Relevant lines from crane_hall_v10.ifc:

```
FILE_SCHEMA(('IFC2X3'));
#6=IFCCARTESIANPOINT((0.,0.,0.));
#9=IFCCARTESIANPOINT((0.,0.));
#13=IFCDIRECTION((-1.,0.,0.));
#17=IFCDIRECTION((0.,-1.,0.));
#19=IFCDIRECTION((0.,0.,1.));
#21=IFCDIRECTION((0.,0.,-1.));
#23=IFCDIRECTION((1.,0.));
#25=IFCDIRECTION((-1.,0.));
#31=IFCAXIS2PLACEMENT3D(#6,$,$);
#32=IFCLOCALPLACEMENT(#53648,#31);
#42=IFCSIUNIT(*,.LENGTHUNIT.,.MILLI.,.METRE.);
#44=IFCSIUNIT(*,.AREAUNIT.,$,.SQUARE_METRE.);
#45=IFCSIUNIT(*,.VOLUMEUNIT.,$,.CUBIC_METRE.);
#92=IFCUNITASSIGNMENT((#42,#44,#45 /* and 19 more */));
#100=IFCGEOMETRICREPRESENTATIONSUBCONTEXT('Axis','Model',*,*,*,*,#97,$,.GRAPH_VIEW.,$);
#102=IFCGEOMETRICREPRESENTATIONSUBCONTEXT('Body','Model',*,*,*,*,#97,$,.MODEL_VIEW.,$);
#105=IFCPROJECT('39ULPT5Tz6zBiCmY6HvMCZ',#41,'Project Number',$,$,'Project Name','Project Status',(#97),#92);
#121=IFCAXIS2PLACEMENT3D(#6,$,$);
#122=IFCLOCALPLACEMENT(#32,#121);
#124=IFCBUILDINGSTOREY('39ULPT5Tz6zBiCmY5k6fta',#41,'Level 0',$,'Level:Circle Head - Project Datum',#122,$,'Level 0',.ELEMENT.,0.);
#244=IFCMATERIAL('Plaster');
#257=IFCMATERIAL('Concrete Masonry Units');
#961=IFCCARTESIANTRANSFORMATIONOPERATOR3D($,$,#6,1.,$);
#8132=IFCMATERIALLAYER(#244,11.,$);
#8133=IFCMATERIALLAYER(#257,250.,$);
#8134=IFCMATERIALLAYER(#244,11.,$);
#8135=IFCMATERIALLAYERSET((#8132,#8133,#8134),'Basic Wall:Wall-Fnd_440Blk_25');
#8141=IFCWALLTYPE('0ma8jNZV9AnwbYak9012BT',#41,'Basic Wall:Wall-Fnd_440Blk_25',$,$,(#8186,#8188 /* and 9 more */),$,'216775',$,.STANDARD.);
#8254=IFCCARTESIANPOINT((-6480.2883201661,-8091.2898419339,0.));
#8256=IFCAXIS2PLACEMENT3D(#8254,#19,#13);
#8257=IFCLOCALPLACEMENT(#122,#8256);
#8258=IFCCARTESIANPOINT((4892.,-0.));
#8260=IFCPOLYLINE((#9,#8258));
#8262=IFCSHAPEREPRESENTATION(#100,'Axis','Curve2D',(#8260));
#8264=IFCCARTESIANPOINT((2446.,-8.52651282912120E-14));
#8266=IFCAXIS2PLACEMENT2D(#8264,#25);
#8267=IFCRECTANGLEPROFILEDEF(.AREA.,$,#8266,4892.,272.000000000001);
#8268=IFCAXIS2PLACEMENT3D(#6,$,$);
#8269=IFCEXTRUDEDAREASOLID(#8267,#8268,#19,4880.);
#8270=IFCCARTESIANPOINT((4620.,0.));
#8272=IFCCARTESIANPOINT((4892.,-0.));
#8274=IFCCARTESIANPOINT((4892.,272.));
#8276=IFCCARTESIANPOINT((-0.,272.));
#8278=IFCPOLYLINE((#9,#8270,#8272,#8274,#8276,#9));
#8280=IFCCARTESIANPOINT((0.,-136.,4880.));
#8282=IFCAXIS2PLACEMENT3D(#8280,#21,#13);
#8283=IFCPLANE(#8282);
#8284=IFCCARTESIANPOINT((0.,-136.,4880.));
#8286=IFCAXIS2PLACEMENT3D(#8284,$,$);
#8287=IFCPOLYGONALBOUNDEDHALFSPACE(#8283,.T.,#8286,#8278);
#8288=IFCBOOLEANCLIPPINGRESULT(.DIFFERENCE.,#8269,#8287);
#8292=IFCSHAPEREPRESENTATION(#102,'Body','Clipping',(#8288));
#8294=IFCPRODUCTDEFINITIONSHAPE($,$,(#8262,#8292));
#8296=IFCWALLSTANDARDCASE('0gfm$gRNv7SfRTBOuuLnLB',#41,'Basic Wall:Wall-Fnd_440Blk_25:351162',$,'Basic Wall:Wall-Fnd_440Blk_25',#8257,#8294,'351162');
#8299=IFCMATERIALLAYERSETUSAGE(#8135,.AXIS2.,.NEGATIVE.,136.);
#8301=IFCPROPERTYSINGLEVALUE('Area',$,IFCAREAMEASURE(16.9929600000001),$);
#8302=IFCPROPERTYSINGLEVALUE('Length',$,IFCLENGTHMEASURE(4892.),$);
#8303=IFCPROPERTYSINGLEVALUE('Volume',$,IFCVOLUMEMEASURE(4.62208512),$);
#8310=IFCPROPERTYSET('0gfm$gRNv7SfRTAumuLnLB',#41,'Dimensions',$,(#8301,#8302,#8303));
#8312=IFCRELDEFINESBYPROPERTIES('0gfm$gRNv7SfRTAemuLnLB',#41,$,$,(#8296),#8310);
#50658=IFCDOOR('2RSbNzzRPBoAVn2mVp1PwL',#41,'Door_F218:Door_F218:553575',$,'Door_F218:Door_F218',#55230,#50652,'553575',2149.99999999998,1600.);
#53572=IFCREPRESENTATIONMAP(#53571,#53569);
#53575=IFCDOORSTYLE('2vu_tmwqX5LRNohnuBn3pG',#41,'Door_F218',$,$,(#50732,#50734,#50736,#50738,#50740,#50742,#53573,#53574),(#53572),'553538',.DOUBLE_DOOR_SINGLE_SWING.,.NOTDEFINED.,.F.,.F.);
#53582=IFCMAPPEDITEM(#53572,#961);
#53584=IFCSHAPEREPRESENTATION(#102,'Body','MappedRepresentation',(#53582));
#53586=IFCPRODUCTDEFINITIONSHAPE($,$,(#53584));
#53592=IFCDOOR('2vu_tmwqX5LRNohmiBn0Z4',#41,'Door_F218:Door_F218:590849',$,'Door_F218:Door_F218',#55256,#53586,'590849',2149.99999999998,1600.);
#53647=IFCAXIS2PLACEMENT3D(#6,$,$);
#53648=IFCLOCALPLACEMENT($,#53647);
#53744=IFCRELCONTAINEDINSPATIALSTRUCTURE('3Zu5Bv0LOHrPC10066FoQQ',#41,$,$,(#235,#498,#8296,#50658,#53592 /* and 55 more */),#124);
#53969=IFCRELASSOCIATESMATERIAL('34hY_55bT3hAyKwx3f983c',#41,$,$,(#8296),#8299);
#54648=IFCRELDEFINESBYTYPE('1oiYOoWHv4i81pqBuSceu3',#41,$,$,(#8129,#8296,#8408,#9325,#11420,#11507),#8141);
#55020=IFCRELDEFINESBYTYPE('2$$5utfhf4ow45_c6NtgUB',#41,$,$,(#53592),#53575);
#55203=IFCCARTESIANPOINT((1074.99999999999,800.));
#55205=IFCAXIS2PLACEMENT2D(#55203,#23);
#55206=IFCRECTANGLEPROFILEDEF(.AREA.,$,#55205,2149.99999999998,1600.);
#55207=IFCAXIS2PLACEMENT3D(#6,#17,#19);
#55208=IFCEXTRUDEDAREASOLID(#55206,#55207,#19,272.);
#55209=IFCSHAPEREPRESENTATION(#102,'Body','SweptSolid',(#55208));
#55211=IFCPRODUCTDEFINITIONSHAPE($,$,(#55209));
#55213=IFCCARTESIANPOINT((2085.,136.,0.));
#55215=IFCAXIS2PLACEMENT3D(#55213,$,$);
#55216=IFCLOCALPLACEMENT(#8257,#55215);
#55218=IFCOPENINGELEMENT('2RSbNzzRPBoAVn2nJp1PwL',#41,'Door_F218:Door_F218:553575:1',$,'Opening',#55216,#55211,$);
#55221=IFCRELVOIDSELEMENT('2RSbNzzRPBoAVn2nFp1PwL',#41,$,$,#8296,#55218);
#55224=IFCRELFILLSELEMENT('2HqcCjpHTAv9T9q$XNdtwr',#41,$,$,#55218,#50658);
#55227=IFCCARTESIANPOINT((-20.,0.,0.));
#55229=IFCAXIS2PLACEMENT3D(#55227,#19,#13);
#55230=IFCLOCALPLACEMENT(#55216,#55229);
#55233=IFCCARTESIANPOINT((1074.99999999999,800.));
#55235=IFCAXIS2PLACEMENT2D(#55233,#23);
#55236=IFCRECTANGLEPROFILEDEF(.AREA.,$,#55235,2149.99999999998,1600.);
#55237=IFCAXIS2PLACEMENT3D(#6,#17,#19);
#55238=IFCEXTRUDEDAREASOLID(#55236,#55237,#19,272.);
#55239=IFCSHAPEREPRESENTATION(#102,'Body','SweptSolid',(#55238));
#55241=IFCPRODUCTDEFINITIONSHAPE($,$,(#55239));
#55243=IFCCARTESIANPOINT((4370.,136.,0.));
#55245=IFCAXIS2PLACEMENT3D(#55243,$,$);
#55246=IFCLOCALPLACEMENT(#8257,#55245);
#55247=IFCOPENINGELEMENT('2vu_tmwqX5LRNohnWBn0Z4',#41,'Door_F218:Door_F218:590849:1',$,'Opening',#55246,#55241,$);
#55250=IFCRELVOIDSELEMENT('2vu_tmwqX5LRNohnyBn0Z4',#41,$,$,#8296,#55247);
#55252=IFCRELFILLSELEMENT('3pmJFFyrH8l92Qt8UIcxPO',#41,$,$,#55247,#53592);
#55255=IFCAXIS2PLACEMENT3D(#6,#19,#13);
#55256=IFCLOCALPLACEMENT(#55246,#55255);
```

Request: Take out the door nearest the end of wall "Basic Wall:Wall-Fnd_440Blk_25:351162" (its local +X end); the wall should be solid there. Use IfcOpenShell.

```python
import ifcopenshell
import ifcopenshell.api.feature
import ifcopenshell.api.pset
import ifcopenshell.api.root
import ifcopenshell.geom
import ifcopenshell.util.element
import ifcopenshell.util.shape
import ifcopenshell.util.unit

model = ifcopenshell.open("crane_hall_v10.ifc")
area_scale = ifcopenshell.util.unit.calculate_unit_scale(model, "AREAUNIT")
volume_scale = ifcopenshell.util.unit.calculate_unit_scale(model, "VOLUMEUNIT")
settings = ifcopenshell.geom.settings()


def volume(element):
    """Net volume in cubic metres, openings subtracted."""
    shape = ifcopenshell.geom.create_shape(settings, element)
    return ifcopenshell.util.shape.get_volume(shape.geometry)


door = model.by_guid("2vu_tmwqX5LRNohmiBn0Z4")
opening = door.FillsVoids[0].RelatingOpeningElement
wall = opening.VoidsElements[0].RelatingBuildingElement
before = volume(wall)

ifcopenshell.api.root.remove_product(model, product=door)
ifcopenshell.api.feature.remove_feature(model, feature=opening)

after = volume(wall)
thickness = 0.272  # wall thickness in metres

# Update the wall's stored quantities.
pset = model.by_id(ifcopenshell.util.element.get_pset(wall, "Dimensions", should_inherit=False)["id"])
ifcopenshell.api.pset.edit_pset(model, pset=pset, properties={
    "Area": model.create_entity("IfcAreaMeasure", after / thickness / area_scale),
    "Volume": model.create_entity("IfcVolumeMeasure", after / volume_scale),
})

print(f"wall volume {before:.3f} -> {after:.3f} m3")

model.write("crane_hall_v10_rev.ifc")
```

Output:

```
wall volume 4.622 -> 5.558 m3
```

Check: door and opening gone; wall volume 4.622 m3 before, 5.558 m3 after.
